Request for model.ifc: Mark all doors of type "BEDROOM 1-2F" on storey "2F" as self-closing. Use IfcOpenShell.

First a look at what the model holds.

```python
import ifcopenshell
import ifcopenshell.util.element

model = ifcopenshell.open("model.ifc")
print(model.schema)
storey = next(s for s in model.by_type("IfcBuildingStorey") if s.Name == "2F")
doors = [e for e in ifcopenshell.util.element.get_decomposition(storey) if e.is_a("IfcDoor")]
seen = {}
for e in doors:
    element_type = ifcopenshell.util.element.get_type(e)
    key = (element_type.Name if element_type != e and element_type else None, ifcopenshell.util.element.get_pset(e, "Pset_DoorCommon", "SelfClosing"))
    seen[key] = seen.get(key, 0) + 1
for (name, value), count in sorted(seen.items(), key=str):
    print(count, "x", name, "|", value)
```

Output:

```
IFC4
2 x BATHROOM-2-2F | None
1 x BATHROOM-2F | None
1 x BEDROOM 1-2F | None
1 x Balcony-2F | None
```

```python
import ifcopenshell
import ifcopenshell.api.pset
import ifcopenshell.util.element

model = ifcopenshell.open("model.ifc")

storey = next(s for s in model.by_type("IfcBuildingStorey") if s.Name == "2F")
doors = [e for e in ifcopenshell.util.element.get_decomposition(storey) if e.is_a("IfcDoor")]

count = 0
for e in doors:
    element_type = ifcopenshell.util.element.get_type(e)
    if element_type in (None, e) or element_type.Name != "BEDROOM 1-2F":
        continue
    # add_pset returns the element's existing set when there is one.
    pset = ifcopenshell.api.pset.add_pset(model, product=e, name="Pset_DoorCommon")
    ifcopenshell.api.pset.edit_pset(model, pset=pset, properties={"SelfClosing": True})
    count += 1

print(count, "doors updated")

model.write("model_v2.ifc")
```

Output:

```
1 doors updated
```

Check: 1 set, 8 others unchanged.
